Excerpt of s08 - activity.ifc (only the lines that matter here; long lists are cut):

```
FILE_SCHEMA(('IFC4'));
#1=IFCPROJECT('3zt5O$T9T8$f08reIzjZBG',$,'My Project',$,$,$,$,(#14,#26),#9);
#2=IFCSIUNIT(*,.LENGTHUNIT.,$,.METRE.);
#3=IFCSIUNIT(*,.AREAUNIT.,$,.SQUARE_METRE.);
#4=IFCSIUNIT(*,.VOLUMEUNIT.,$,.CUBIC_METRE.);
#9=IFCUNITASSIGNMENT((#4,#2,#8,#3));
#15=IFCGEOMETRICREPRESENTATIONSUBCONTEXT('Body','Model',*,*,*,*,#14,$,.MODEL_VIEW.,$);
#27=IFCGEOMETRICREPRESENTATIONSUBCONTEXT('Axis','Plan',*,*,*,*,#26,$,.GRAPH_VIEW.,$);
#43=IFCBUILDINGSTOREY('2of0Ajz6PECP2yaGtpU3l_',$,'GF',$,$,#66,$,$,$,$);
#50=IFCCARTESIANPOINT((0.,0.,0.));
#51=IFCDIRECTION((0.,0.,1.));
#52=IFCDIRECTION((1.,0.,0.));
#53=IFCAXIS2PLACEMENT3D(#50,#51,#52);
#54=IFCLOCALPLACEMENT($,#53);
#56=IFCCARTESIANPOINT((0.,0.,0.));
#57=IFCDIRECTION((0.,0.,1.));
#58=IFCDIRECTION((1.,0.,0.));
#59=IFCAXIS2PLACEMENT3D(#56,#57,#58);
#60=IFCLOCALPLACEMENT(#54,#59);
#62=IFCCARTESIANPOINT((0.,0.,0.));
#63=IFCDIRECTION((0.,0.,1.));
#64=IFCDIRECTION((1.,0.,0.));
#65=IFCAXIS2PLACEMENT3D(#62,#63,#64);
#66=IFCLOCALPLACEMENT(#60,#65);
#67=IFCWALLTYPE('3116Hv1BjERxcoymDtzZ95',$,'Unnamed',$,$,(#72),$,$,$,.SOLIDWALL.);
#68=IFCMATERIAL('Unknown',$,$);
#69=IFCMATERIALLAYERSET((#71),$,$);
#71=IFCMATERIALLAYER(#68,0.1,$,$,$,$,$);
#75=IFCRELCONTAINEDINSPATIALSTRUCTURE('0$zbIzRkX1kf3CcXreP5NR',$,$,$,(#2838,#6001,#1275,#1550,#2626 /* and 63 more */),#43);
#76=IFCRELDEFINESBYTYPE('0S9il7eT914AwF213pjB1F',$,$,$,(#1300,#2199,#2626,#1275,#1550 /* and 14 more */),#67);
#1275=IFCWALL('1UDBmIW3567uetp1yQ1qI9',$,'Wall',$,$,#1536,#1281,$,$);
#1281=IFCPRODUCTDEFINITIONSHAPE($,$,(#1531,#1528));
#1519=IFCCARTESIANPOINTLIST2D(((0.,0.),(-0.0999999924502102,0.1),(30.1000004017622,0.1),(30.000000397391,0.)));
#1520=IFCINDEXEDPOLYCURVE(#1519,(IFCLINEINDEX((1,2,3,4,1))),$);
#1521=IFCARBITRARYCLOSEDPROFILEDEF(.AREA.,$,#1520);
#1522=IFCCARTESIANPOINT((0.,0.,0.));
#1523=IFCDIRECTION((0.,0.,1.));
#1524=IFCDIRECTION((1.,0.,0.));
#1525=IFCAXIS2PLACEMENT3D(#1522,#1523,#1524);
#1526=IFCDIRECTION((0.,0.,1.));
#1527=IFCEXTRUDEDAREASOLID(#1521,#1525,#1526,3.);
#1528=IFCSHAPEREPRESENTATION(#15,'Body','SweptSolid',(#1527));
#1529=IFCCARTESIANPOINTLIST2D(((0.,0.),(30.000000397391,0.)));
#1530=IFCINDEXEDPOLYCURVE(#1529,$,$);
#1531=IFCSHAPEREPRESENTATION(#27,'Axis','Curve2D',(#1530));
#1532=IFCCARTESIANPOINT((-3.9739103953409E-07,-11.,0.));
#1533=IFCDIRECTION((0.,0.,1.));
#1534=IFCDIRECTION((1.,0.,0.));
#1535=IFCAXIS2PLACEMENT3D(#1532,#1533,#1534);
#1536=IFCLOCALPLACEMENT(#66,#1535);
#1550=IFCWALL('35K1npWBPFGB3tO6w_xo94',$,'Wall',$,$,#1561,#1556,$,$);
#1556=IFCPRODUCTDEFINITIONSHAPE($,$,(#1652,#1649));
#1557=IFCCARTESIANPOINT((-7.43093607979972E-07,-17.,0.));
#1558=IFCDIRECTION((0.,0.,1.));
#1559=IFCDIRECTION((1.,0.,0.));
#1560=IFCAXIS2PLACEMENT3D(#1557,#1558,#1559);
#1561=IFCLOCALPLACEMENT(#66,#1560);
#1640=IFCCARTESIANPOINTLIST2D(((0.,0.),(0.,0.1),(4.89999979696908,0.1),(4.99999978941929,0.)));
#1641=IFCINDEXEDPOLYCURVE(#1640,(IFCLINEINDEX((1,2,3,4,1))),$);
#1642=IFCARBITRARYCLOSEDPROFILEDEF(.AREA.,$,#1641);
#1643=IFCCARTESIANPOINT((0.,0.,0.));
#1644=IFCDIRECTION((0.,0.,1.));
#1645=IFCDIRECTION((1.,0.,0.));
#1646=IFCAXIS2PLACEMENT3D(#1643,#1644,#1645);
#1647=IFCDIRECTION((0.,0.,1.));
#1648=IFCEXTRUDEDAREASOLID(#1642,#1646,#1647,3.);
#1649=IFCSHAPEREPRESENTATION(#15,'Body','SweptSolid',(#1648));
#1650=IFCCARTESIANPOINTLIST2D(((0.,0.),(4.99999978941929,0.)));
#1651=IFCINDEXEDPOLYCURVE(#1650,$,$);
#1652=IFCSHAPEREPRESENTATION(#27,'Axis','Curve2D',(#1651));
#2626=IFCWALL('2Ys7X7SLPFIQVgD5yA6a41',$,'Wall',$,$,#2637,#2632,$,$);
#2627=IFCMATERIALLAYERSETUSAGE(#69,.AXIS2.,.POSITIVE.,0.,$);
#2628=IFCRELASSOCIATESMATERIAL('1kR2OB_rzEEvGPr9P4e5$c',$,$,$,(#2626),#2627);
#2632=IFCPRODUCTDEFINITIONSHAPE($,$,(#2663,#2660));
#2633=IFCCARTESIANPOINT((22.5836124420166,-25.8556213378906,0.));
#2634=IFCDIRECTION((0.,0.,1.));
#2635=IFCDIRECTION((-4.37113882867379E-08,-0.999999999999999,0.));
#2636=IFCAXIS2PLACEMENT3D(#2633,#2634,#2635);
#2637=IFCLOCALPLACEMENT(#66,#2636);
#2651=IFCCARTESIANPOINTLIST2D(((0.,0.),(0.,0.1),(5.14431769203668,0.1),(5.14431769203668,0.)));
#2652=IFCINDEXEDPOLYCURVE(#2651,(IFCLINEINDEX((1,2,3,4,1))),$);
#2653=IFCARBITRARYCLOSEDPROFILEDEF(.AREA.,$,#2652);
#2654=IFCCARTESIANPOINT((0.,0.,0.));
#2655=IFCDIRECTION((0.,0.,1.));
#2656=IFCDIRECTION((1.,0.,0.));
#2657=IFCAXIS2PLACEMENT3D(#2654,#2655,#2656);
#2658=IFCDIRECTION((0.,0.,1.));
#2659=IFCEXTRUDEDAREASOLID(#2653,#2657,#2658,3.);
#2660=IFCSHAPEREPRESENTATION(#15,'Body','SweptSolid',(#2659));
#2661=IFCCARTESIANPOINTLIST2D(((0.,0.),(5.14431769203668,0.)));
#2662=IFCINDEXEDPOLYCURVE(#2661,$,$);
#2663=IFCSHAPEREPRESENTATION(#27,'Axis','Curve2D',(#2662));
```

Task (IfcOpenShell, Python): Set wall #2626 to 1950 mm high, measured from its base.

```python
import ifcopenshell
import ifcopenshell.geom
import ifcopenshell.util.representation
import ifcopenshell.util.shape
import ifcopenshell.util.unit

model = ifcopenshell.open("s08 - activity.ifc")
unit_scale = ifcopenshell.util.unit.calculate_unit_scale(model)
settings = ifcopenshell.geom.settings()


def volume(element):
    """Net volume in cubic metres, openings subtracted."""
    shape = ifcopenshell.geom.create_shape(settings, element)
    return ifcopenshell.util.shape.get_volume(shape.geometry)


wall = model.by_guid("2Ys7X7SLPFIQVgD5yA6a41")
before = volume(wall)

body = ifcopenshell.util.representation.get_representation(wall, "Model", "Body")
solid = body.Items[0]
old_height = solid.Depth
solid.Depth = 1.95 / unit_scale
after = volume(wall)

print(f"height {old_height:g} -> {solid.Depth:g}, volume {before:.3f} -> {after:.3f} m3")

model.write("s08 - activity-out.ifc")
```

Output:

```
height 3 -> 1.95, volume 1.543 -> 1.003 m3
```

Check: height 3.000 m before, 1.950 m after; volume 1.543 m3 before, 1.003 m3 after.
